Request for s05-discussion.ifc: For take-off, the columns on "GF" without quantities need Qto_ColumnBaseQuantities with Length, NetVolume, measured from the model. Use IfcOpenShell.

First a look at what the model holds.

```python
import ifcopenshell
import ifcopenshell.util.element
import ifcopenshell.util.unit

model = ifcopenshell.open("s05-discussion.ifc")
print(model.schema)
for unit_type in ("LENGTHUNIT", "AREAUNIT", "VOLUMEUNIT"):
    print(unit_type, ifcopenshell.util.unit.calculate_unit_scale(model, unit_type))
storey = next(s for s in model.by_type("IfcBuildingStorey") if s.Name == "GF")
columns = [e for e in ifcopenshell.util.element.get_decomposition(storey) if e.is_a("IfcColumn")]
for e in sorted(columns, key=lambda e: e.id()):
    print(e.id(), e.is_a(), e.Name, list(ifcopenshell.util.element.get_psets(e, qtos_only=True)), sep=" | ")
```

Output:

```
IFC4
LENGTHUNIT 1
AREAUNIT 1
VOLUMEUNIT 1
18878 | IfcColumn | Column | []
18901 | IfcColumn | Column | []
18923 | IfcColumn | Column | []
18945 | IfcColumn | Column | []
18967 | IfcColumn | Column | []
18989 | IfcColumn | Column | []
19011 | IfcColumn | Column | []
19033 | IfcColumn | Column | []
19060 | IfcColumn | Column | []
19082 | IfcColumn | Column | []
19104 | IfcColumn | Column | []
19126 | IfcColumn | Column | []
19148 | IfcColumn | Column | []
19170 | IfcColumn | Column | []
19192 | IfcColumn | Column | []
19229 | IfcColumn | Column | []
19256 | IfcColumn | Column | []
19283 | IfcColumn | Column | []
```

```python
import ifcopenshell
import ifcopenshell.api.pset
import ifcopenshell.geom
import ifcopenshell.util.element
import ifcopenshell.util.shape
import ifcopenshell.util.unit

model = ifcopenshell.open("s05-discussion.ifc")
unit_scale = ifcopenshell.util.unit.calculate_unit_scale(model)
volume_scale = ifcopenshell.util.unit.calculate_unit_scale(model, "VOLUMEUNIT")
settings = ifcopenshell.geom.settings()

storey = next(s for s in model.by_type("IfcBuildingStorey") if s.Name == "GF")
columns = [e for e in ifcopenshell.util.element.get_decomposition(storey) if e.is_a("IfcColumn")]

for e in sorted(columns, key=lambda e: e.id()):
    if ifcopenshell.util.element.get_psets(e, qtos_only=True, should_inherit=False):
        continue
    # Geometry comes back in metres, in the element's own axes.
    shape = ifcopenshell.geom.create_shape(settings, e)
    values = {
        "Length": ifcopenshell.util.shape.get_z(shape.geometry) / unit_scale,
        "NetVolume": ifcopenshell.util.shape.get_volume(shape.geometry) / volume_scale,
    }
    qto = ifcopenshell.api.pset.add_qto(model, product=e, name="Qto_ColumnBaseQuantities")
    ifcopenshell.api.pset.edit_qto(model, qto=qto, properties=values)
    print(e.id(), {k: round(v, 3) for k, v in values.items()})

model.write("s05-discussion_rev.ifc")
```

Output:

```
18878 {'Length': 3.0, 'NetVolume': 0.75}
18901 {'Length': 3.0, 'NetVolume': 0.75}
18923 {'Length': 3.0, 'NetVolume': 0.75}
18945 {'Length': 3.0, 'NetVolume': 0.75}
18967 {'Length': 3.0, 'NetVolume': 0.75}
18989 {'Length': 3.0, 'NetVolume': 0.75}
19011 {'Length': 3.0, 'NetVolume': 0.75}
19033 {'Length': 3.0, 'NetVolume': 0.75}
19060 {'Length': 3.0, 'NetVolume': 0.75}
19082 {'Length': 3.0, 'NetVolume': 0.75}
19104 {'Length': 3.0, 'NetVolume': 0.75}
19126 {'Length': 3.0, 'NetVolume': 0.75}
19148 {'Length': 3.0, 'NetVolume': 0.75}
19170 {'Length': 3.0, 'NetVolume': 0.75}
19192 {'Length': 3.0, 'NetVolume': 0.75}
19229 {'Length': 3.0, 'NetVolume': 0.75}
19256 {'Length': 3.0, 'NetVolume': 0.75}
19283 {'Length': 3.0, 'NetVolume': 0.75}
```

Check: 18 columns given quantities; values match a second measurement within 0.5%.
